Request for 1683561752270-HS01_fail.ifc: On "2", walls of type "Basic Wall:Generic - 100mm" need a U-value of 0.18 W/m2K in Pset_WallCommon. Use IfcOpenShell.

First a look at what the model holds.

```python
import ifcopenshell
import ifcopenshell.util.element

model = ifcopenshell.open("1683561752270-HS01_fail.ifc")
print(model.schema)
storey = next(s for s in model.by_type("IfcBuildingStorey") if s.Name == "2")
walls = [e for e in ifcopenshell.util.element.get_decomposition(storey) if e.is_a("IfcWall")]
seen = {}
for e in walls:
    element_type = ifcopenshell.util.element.get_type(e)
    key = (element_type.Name if element_type != e and element_type else None, ifcopenshell.util.element.get_pset(e, "Pset_WallCommon", "ThermalTransmittance"))
    seen[key] = seen.get(key, 0) + 1
for (name, value), count in sorted(seen.items(), key=str):
    print(count, "x", name, "|", value)
```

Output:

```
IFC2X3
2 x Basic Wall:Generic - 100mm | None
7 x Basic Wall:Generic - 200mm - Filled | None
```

```python
import ifcopenshell
import ifcopenshell.api.pset
import ifcopenshell.util.element

model = ifcopenshell.open("1683561752270-HS01_fail.ifc")

storey = next(s for s in model.by_type("IfcBuildingStorey") if s.Name == "2")
walls = [e for e in ifcopenshell.util.element.get_decomposition(storey) if e.is_a("IfcWall")]

count = 0
for e in walls:
    element_type = ifcopenshell.util.element.get_type(e)
    if element_type in (None, e) or element_type.Name != "Basic Wall:Generic - 100mm":
        continue
    # add_pset returns the element's existing set when there is one.
    pset = ifcopenshell.api.pset.add_pset(model, product=e, name="Pset_WallCommon")
    ifcopenshell.api.pset.edit_pset(model, pset=pset, properties={"ThermalTransmittance": 0.18})
    count += 1

print(count, "walls updated")

model.write("1683561752270-HS01_fail_v2.ifc")
```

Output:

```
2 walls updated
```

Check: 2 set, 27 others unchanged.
